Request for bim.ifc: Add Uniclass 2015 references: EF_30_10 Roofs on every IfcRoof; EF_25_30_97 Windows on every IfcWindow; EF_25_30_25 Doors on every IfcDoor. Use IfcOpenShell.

First a look at what the model holds.

```python
import ifcopenshell

model = ifcopenshell.open("bim.ifc")
print(model.schema)
print("classifications:", [c.Name for c in model.by_type("IfcClassification")])
for ifc_class in ("IfcDoor", "IfcRoof", "IfcStair", "IfcWall", "IfcWindow"):
    print(ifc_class, len(model.by_type(ifc_class)))
```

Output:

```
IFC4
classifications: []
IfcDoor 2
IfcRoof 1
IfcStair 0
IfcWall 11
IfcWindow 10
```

```python
import ifcopenshell
import ifcopenshell.api.classification

model = ifcopenshell.open("bim.ifc")

system = ifcopenshell.api.classification.add_classification(model, classification="Uniclass 2015")

codes = {
    "IfcRoof": ("EF_30_10", "Roofs"),
    "IfcWindow": ("EF_25_30_97", "Windows"),
    "IfcDoor": ("EF_25_30_25", "Doors"),
}
for ifc_class, (code, name) in codes.items():
    products = model.by_type(ifc_class)
    ifcopenshell.api.classification.add_reference(
        model, products=products, classification=system, identification=code, name=name
    )
    print(code, len(products))

model.write("bim-out.ifc")
```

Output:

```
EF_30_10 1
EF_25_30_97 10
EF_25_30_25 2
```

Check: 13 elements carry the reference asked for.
